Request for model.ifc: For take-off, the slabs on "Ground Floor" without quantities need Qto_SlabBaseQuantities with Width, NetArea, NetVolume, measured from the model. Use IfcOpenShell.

First a look at what the model holds.

```python
import ifcopenshell
import ifcopenshell.util.element
import ifcopenshell.util.unit

model = ifcopenshell.open("model.ifc")
print(model.schema)
for unit_type in ("LENGTHUNIT", "AREAUNIT", "VOLUMEUNIT"):
    print(unit_type, ifcopenshell.util.unit.calculate_unit_scale(model, unit_type))
storey = next(s for s in model.by_type("IfcBuildingStorey") if s.Name == "Ground Floor")
slabs = [e for e in ifcopenshell.util.element.get_decomposition(storey) if e.is_a("IfcSlab")]
for e in sorted(slabs, key=lambda e: e.id()):
    print(e.id(), e.is_a(), e.Name, list(ifcopenshell.util.element.get_psets(e, qtos_only=True)), sep=" | ")
```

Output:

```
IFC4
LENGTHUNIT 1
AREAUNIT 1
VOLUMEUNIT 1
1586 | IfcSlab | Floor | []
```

```python
import ifcopenshell
import ifcopenshell.api.pset
import ifcopenshell.geom
import ifcopenshell.util.element
import ifcopenshell.util.shape
import ifcopenshell.util.unit

model = ifcopenshell.open("model.ifc")
unit_scale = ifcopenshell.util.unit.calculate_unit_scale(model)
area_scale = ifcopenshell.util.unit.calculate_unit_scale(model, "AREAUNIT")
volume_scale = ifcopenshell.util.unit.calculate_unit_scale(model, "VOLUMEUNIT")
settings = ifcopenshell.geom.settings()

storey = next(s for s in model.by_type("IfcBuildingStorey") if s.Name == "Ground Floor")
slabs = [e for e in ifcopenshell.util.element.get_decomposition(storey) if e.is_a("IfcSlab")]

for e in sorted(slabs, key=lambda e: e.id()):
    if ifcopenshell.util.element.get_psets(e, qtos_only=True, should_inherit=False):
        continue
    # Geometry comes back in metres, in the element's own axes.
    shape = ifcopenshell.geom.create_shape(settings, e)
    values = {
        "Width": ifcopenshell.util.shape.get_z(shape.geometry) / unit_scale,
        "NetArea": ifcopenshell.util.shape.get_footprint_area(shape.geometry) / area_scale,
        "NetVolume": ifcopenshell.util.shape.get_volume(shape.geometry) / volume_scale,
    }
    qto = ifcopenshell.api.pset.add_qto(model, product=e, name="Qto_SlabBaseQuantities")
    ifcopenshell.api.pset.edit_qto(model, qto=qto, properties=values)
    print(e.id(), {k: round(v, 3) for k, v in values.items()})

model.write("model_v2.ifc")
```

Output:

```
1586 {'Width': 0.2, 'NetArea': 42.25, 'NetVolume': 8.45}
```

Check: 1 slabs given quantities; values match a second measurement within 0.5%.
